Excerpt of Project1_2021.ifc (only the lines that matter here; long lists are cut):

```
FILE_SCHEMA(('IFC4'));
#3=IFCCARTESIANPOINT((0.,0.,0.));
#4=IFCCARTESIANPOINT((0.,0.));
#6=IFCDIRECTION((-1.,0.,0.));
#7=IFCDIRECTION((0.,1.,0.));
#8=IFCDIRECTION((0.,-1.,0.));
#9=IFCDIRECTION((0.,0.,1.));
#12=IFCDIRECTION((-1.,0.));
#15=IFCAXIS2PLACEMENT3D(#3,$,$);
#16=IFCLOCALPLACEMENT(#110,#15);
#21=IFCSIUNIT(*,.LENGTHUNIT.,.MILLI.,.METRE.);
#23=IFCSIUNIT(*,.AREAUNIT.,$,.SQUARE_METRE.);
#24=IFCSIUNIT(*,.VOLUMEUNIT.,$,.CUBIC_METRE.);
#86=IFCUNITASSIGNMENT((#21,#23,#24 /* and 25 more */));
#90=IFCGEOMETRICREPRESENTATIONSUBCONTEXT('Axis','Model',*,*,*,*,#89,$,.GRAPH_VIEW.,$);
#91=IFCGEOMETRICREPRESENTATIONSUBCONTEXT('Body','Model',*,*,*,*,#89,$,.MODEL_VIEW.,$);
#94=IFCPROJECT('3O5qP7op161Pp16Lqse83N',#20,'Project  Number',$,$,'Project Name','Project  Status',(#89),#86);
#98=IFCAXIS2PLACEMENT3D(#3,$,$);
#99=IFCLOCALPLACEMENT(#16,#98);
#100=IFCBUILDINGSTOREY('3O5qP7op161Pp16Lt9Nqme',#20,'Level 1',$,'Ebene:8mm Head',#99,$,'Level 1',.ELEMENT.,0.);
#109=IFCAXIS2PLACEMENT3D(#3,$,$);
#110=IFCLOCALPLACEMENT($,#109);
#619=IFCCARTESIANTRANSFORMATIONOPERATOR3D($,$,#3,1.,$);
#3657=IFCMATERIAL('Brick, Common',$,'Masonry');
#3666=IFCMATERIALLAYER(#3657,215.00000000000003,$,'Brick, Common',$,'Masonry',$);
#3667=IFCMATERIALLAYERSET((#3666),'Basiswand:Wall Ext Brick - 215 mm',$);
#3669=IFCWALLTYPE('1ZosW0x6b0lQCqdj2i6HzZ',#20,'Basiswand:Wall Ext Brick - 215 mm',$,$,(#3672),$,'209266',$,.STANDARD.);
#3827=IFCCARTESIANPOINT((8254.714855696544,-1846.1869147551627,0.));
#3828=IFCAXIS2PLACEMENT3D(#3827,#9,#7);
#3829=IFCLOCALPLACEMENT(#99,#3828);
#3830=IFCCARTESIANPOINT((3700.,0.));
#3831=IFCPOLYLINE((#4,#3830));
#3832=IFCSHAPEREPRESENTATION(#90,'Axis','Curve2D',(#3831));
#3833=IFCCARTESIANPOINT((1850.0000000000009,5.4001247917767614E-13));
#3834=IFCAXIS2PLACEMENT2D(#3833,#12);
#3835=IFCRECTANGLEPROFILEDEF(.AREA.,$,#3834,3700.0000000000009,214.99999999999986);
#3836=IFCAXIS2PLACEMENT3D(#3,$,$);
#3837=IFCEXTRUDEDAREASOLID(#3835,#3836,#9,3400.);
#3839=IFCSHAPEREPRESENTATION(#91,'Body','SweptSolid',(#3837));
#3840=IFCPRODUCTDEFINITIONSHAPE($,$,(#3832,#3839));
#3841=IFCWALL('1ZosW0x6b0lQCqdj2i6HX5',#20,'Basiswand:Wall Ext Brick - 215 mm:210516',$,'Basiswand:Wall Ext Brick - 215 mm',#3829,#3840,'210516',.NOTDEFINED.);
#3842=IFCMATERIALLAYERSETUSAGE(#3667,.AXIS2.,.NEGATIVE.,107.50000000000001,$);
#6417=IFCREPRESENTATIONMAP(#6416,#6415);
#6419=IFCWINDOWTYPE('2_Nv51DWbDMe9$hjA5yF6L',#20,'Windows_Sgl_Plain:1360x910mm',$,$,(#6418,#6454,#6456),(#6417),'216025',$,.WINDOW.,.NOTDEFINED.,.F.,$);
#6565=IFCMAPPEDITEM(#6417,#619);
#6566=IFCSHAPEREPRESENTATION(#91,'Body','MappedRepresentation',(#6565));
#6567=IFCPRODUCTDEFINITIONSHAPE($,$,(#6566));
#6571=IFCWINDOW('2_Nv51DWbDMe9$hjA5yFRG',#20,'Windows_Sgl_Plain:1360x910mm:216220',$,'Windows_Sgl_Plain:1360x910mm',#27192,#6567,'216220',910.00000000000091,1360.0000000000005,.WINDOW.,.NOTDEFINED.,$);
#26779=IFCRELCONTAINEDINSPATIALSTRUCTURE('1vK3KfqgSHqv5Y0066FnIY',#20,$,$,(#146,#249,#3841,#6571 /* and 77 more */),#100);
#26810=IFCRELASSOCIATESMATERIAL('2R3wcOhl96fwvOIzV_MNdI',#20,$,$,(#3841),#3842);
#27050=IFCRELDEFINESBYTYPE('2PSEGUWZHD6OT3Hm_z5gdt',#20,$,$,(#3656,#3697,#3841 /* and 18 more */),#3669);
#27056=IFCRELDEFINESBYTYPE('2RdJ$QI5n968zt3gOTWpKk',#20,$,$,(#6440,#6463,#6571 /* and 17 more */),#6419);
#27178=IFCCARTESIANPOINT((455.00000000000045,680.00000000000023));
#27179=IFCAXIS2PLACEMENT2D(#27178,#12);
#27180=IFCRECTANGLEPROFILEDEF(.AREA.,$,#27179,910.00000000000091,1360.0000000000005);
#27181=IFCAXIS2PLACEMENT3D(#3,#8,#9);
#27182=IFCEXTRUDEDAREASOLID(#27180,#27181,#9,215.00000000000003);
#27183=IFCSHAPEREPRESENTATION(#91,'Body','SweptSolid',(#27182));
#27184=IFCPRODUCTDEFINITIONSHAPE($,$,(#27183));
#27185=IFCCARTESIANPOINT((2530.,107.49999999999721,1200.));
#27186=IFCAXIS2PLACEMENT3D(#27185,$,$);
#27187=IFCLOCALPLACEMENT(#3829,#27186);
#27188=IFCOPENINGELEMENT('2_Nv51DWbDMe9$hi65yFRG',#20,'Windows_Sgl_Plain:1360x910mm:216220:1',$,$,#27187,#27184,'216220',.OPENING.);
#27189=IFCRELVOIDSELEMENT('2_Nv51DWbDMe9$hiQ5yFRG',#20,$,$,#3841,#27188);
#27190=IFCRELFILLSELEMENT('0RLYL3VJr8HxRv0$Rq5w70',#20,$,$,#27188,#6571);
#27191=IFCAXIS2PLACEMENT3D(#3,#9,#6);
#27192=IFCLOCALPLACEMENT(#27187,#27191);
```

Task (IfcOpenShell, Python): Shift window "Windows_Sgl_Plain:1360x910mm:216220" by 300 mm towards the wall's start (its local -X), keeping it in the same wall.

```python
import ifcopenshell
import ifcopenshell.api.geometry
import ifcopenshell.util.placement
import ifcopenshell.util.unit

model = ifcopenshell.open("Project1_2021.ifc")
unit_scale = ifcopenshell.util.unit.calculate_unit_scale(model)

window = model.by_guid("2_Nv51DWbDMe9$hjA5yFRG")
opening = window.FillsVoids[0].RelatingOpeningElement
wall = opening.VoidsElements[0].RelatingBuildingElement

wall_matrix = ifcopenshell.util.placement.get_local_placement(wall.ObjectPlacement)
shift = wall_matrix[:3, 0] * -0.3 / unit_scale
before = ifcopenshell.util.placement.get_local_placement(window.ObjectPlacement)[:3, 3].copy()

# The window is placed relative to its opening, so it follows when the opening moves.
matrix = ifcopenshell.util.placement.get_local_placement(opening.ObjectPlacement)
matrix[:3, 3] += shift
ifcopenshell.api.geometry.edit_object_placement(
    model, product=opening, matrix=matrix, is_si=False, should_transform_children=True
)

after = ifcopenshell.util.placement.get_local_placement(window.ObjectPlacement)[:3, 3]
print("window moved by", (after - before).round(3) + 0.0)

model.write("Project1_2021-out.ifc")
```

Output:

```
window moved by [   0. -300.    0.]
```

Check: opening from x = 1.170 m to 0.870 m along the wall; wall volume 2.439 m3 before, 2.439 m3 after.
